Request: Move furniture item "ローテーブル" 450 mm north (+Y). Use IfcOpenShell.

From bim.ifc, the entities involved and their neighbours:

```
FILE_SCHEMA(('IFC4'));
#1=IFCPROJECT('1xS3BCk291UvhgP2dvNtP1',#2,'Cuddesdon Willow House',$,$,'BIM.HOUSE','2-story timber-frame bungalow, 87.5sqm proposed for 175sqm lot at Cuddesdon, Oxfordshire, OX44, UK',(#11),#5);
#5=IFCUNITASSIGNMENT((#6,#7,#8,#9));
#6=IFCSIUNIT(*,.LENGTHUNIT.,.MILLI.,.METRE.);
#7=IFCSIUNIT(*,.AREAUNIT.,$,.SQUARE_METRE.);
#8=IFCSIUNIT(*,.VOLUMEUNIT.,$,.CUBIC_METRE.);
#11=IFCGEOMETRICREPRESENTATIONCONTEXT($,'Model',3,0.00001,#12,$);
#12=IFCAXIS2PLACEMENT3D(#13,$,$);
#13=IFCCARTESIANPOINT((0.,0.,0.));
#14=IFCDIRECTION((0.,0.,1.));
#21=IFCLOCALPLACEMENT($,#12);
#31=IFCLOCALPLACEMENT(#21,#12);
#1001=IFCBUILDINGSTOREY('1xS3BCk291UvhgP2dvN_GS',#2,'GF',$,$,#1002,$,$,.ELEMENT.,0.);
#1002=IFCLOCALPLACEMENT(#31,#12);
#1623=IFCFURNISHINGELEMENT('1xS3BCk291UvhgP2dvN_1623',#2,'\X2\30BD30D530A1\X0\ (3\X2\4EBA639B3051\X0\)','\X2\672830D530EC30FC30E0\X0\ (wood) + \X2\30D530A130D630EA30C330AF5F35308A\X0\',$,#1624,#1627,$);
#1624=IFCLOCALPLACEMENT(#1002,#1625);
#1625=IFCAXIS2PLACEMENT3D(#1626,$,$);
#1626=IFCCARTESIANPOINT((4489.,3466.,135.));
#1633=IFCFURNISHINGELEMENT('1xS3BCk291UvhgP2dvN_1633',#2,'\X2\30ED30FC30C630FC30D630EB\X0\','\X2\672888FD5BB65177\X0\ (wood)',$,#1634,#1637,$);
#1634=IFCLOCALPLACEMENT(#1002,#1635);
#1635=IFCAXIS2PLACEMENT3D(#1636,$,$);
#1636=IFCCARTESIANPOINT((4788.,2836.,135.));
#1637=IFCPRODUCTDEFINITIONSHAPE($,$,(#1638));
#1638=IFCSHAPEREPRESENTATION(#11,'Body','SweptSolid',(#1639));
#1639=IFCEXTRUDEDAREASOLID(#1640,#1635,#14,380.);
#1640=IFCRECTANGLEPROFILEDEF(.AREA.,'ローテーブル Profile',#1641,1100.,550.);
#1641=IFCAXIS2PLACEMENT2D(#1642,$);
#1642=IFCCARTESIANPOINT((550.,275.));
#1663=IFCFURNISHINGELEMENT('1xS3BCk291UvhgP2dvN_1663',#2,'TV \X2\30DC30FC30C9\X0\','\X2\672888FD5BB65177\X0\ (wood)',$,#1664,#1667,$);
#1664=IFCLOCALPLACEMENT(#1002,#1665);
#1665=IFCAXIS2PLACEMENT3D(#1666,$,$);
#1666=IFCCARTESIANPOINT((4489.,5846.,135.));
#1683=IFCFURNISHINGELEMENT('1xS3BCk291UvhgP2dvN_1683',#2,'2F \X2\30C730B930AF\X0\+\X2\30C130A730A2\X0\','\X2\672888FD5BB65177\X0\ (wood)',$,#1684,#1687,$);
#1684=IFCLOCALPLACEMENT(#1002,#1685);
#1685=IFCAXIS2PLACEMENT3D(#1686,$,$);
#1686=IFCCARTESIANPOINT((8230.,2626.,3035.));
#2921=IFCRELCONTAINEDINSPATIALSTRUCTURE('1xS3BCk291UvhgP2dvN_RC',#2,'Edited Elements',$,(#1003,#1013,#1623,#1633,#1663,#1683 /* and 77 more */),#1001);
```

```python
import ifcopenshell
import ifcopenshell.api.geometry
import ifcopenshell.util.placement
import ifcopenshell.util.unit

model = ifcopenshell.open("bim.ifc")
unit_scale = ifcopenshell.util.unit.calculate_unit_scale(model)

item = model.by_guid("1xS3BCk291UvhgP2dvN_1633")
matrix = ifcopenshell.util.placement.get_local_placement(item.ObjectPlacement)
matrix[1, 3] += 0.45 / unit_scale
ifcopenshell.api.geometry.edit_object_placement(model, product=item, matrix=matrix, is_si=False)

print(ifcopenshell.util.placement.get_local_placement(item.ObjectPlacement).round(3) + 0.0)

model.write("bim_updated.ifc")
```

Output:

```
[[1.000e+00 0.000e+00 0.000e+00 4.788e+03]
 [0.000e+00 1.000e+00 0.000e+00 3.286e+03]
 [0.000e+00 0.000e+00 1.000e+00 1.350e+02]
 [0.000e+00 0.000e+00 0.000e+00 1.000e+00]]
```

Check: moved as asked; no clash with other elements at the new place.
